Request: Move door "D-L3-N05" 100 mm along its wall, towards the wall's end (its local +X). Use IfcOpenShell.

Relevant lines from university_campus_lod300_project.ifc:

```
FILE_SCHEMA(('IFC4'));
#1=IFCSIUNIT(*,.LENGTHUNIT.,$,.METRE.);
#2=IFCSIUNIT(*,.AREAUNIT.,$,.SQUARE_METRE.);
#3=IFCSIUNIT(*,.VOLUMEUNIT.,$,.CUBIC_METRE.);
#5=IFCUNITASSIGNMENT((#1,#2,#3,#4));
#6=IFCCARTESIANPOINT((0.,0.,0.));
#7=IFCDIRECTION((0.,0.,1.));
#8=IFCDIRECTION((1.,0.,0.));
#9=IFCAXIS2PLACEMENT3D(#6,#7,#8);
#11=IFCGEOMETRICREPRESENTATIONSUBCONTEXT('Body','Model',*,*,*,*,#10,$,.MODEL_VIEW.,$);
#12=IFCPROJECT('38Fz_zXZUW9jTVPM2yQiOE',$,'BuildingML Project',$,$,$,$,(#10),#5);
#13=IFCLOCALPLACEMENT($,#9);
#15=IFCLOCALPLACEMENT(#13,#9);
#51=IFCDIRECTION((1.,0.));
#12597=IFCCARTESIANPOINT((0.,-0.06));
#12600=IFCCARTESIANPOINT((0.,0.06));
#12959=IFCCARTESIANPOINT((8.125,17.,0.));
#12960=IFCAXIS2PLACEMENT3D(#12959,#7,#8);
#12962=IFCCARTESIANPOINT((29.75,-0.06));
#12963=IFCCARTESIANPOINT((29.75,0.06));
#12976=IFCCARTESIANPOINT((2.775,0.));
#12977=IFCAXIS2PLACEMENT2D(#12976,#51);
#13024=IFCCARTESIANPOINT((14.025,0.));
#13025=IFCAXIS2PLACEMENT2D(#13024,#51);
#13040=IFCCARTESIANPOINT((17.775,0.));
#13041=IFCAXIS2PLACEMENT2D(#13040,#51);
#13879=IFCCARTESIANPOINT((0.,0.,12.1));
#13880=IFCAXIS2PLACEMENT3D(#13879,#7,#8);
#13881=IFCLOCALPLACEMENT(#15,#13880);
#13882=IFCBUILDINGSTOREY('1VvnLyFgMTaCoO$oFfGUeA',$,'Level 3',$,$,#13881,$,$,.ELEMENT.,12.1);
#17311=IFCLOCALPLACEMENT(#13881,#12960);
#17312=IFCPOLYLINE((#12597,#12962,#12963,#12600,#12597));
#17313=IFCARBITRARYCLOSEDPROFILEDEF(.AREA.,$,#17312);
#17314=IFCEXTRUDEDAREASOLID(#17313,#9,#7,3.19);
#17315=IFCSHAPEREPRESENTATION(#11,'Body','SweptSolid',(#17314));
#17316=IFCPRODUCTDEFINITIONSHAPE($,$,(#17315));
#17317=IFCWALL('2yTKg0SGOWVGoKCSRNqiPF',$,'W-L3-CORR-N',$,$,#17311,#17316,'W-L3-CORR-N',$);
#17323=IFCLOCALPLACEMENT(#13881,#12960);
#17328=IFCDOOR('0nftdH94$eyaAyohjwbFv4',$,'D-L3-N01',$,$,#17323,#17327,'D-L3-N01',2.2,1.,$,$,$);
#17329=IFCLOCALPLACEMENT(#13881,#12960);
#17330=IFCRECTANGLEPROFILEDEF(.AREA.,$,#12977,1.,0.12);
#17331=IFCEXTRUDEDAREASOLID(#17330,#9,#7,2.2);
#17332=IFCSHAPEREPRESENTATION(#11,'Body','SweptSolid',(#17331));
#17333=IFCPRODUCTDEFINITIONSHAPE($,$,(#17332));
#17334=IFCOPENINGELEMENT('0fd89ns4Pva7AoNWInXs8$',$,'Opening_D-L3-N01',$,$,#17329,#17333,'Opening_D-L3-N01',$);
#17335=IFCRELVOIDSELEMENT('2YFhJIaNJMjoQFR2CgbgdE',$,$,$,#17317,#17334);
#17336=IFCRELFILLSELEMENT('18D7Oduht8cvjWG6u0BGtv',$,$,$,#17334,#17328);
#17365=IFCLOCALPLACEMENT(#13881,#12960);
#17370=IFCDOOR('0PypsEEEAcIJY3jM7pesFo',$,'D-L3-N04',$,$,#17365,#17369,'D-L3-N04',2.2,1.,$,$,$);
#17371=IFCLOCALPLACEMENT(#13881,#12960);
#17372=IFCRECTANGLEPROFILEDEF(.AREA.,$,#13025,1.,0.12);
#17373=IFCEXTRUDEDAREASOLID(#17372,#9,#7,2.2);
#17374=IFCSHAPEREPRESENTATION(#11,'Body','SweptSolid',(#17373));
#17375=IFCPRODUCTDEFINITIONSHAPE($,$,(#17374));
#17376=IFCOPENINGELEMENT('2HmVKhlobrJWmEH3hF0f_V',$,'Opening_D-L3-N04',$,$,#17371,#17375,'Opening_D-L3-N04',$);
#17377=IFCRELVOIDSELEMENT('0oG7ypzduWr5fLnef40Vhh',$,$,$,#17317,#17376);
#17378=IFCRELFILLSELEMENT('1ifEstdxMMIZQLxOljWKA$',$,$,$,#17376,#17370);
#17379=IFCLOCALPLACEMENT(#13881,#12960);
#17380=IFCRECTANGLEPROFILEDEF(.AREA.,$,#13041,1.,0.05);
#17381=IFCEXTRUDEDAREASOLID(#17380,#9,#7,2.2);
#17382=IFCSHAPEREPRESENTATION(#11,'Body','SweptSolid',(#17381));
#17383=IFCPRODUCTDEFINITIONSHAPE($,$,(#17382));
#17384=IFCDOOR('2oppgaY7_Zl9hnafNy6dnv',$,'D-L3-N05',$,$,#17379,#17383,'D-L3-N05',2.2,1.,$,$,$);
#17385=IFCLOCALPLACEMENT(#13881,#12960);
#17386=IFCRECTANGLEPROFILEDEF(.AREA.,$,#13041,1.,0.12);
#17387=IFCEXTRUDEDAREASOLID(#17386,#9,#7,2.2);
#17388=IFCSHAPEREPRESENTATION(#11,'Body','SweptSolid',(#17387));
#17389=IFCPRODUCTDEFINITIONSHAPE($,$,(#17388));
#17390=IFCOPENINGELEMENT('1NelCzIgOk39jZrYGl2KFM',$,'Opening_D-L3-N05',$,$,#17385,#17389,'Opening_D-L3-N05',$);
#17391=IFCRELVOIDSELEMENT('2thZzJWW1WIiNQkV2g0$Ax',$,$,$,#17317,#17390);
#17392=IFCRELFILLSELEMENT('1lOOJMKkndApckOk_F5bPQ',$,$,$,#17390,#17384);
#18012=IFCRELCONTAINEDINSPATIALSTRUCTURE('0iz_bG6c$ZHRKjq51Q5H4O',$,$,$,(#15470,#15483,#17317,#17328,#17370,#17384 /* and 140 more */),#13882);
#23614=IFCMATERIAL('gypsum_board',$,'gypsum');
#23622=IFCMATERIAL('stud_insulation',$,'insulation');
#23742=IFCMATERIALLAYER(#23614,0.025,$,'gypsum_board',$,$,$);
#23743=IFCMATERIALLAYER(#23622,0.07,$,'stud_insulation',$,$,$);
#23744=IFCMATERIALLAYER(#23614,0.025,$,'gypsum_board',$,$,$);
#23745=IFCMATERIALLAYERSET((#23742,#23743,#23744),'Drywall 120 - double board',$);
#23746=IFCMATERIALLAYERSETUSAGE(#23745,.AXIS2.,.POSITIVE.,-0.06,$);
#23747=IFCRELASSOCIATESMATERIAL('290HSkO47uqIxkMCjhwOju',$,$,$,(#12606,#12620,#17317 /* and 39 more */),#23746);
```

```python
import ifcopenshell
import ifcopenshell.api.geometry
import ifcopenshell.util.placement
import ifcopenshell.util.unit

model = ifcopenshell.open("university_campus_lod300_project.ifc")
unit_scale = ifcopenshell.util.unit.calculate_unit_scale(model)

door = model.by_guid("2oppgaY7_Zl9hnafNy6dnv")
opening = door.FillsVoids[0].RelatingOpeningElement
wall = opening.VoidsElements[0].RelatingBuildingElement

wall_matrix = ifcopenshell.util.placement.get_local_placement(wall.ObjectPlacement)
shift = wall_matrix[:3, 0] * 0.1 / unit_scale
before = ifcopenshell.util.placement.get_local_placement(door.ObjectPlacement)[:3, 3].copy()

# The door is not placed relative to its opening, so move both.
for product in (opening, door):
    matrix = ifcopenshell.util.placement.get_local_placement(product.ObjectPlacement)
    matrix[:3, 3] += shift
    ifcopenshell.api.geometry.edit_object_placement(model, product=product, matrix=matrix, is_si=False)

after = ifcopenshell.util.placement.get_local_placement(door.ObjectPlacement)[:3, 3]
print("door moved by", (after - before).round(3) + 0.0)

model.write("university_campus_lod300_project_rev.ifc")
```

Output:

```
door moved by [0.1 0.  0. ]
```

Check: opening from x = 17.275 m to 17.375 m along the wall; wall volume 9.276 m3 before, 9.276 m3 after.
